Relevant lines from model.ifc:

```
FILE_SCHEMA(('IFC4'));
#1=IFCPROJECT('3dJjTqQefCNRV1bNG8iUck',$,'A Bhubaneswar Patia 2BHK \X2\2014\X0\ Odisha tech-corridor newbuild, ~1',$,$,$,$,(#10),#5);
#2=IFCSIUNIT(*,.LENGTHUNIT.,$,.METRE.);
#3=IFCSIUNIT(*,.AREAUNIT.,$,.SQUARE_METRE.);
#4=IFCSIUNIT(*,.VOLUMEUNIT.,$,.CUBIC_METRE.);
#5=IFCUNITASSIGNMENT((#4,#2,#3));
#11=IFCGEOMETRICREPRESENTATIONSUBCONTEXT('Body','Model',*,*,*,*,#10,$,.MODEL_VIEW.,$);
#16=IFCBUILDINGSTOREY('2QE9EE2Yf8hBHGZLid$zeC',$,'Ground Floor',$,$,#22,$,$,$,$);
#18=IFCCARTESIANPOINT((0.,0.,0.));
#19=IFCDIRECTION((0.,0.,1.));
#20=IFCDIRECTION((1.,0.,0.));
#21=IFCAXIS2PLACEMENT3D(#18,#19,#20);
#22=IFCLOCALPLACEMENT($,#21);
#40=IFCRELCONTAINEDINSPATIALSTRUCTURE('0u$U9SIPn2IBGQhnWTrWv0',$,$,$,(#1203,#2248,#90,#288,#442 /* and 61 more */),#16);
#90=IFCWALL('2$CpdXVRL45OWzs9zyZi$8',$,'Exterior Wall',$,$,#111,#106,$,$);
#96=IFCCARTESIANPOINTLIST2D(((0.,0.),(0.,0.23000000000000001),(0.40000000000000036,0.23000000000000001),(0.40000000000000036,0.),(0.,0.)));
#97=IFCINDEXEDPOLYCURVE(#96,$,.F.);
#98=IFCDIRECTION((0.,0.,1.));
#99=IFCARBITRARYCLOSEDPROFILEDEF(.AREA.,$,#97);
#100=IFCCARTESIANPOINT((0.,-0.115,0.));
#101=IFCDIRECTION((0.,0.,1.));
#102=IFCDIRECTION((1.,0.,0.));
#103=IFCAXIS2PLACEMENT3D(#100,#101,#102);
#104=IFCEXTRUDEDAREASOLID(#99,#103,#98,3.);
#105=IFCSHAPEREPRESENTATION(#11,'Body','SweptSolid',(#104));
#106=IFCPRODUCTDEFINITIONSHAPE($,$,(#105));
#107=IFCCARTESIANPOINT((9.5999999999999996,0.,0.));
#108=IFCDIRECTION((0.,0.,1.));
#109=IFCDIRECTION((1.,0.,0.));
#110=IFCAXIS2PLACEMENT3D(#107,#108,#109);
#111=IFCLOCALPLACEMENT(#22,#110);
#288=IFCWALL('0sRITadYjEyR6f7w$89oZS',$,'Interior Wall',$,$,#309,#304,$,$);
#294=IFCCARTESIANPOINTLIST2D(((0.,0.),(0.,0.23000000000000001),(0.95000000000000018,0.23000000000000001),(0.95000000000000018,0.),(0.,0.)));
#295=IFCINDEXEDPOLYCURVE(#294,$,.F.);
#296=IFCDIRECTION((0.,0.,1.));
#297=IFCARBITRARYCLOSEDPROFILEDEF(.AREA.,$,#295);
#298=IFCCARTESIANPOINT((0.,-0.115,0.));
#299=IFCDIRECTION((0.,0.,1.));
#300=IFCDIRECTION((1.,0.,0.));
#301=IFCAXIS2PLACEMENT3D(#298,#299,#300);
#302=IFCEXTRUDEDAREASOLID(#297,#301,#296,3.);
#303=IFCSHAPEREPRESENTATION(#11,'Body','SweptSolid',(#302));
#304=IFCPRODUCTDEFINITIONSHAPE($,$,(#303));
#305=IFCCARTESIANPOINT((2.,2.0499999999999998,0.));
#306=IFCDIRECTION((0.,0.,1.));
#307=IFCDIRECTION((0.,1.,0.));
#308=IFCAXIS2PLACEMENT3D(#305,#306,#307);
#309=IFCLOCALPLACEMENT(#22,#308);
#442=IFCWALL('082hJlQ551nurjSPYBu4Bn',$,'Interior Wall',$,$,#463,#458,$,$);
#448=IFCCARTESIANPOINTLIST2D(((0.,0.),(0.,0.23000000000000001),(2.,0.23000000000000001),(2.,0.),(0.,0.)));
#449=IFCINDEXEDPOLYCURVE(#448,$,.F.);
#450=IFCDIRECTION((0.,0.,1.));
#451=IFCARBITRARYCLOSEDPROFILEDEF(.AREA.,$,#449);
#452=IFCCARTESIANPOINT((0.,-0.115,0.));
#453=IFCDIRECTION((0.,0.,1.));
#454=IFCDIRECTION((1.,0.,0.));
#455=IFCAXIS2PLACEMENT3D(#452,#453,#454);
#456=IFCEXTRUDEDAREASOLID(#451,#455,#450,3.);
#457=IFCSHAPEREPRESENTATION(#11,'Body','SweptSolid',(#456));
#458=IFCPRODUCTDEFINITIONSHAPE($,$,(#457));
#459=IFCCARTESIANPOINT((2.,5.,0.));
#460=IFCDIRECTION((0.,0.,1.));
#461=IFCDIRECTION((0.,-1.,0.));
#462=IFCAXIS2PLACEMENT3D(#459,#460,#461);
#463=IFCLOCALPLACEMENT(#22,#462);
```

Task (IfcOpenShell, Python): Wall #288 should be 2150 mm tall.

```python
import ifcopenshell
import ifcopenshell.geom
import ifcopenshell.util.representation
import ifcopenshell.util.shape
import ifcopenshell.util.unit

model = ifcopenshell.open("model.ifc")
unit_scale = ifcopenshell.util.unit.calculate_unit_scale(model)
settings = ifcopenshell.geom.settings()


def volume(element):
    """Net volume in cubic metres, openings subtracted."""
    shape = ifcopenshell.geom.create_shape(settings, element)
    return ifcopenshell.util.shape.get_volume(shape.geometry)


wall = model.by_guid("0sRITadYjEyR6f7w$89oZS")
before = volume(wall)

body = ifcopenshell.util.representation.get_representation(wall, "Model", "Body")
solid = body.Items[0]
old_height = solid.Depth
solid.Depth = 2.15 / unit_scale
after = volume(wall)

print(f"height {old_height:g} -> {solid.Depth:g}, volume {before:.3f} -> {after:.3f} m3")

model.write("model_edited.ifc")
```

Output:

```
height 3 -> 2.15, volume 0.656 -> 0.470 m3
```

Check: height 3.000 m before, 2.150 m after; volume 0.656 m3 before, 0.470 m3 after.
